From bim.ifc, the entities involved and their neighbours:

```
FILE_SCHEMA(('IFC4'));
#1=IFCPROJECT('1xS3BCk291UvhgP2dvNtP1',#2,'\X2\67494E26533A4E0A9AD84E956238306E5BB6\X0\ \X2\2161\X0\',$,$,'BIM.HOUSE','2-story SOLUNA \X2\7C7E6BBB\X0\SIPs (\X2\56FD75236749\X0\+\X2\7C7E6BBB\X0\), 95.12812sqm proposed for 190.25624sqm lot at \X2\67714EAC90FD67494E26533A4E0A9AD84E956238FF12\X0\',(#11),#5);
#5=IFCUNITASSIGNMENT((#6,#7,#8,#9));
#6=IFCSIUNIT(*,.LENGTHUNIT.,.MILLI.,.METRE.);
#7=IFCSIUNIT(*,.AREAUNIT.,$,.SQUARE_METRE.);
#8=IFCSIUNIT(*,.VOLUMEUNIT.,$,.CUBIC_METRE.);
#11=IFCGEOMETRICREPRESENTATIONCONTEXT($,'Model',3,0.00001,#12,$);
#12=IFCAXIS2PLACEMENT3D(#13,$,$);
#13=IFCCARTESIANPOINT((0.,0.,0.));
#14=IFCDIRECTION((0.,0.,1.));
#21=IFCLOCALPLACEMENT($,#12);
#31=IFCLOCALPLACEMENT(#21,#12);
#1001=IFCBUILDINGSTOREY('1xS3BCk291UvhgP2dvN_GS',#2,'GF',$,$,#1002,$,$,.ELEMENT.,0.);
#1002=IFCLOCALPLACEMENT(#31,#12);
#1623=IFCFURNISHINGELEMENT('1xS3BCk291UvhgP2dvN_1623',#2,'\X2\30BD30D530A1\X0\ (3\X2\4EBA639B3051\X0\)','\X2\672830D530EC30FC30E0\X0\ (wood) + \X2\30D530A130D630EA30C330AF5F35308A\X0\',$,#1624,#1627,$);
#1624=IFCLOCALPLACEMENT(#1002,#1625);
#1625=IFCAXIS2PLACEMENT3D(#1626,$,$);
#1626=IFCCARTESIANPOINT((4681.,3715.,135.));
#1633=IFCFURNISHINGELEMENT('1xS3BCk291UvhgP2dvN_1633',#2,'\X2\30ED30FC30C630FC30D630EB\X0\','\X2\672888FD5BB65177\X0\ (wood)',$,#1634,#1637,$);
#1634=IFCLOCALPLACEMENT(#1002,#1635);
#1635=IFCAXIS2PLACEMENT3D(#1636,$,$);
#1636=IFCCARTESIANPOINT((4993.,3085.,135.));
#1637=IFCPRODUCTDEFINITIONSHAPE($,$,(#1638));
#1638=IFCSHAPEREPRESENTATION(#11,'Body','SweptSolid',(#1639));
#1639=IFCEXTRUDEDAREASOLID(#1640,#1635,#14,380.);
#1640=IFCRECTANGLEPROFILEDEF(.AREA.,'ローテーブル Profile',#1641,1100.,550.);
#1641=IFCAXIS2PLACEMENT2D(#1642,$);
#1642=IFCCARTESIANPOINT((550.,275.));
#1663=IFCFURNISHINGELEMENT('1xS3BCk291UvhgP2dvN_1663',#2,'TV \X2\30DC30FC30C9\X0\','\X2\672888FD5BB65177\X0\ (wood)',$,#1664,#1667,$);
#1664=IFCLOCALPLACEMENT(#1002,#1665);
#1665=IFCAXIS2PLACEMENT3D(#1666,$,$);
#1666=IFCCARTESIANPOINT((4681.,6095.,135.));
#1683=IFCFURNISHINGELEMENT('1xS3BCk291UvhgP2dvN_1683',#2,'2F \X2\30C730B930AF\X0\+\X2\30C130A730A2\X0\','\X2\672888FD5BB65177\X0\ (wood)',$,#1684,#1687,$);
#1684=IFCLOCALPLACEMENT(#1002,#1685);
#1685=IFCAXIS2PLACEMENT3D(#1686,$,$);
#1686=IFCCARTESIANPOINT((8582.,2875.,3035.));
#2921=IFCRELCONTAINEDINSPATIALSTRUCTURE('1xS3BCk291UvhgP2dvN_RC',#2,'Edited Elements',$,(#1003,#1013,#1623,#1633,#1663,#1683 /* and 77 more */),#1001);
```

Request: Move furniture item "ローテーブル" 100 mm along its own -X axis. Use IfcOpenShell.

```python
import ifcopenshell
import ifcopenshell.api.geometry
import ifcopenshell.util.placement
import ifcopenshell.util.unit

model = ifcopenshell.open("bim.ifc")
unit_scale = ifcopenshell.util.unit.calculate_unit_scale(model)

item = model.by_guid("1xS3BCk291UvhgP2dvN_1633")
matrix = ifcopenshell.util.placement.get_local_placement(item.ObjectPlacement)
matrix[:3, 3] -= matrix[:3, 0] * 0.1 / unit_scale
ifcopenshell.api.geometry.edit_object_placement(model, product=item, matrix=matrix, is_si=False)

print(ifcopenshell.util.placement.get_local_placement(item.ObjectPlacement).round(3) + 0.0)

model.write("bim-out.ifc")
```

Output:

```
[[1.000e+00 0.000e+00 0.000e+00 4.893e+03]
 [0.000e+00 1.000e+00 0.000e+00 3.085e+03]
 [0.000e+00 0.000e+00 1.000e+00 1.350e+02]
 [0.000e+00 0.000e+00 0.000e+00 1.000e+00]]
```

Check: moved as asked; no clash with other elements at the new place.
